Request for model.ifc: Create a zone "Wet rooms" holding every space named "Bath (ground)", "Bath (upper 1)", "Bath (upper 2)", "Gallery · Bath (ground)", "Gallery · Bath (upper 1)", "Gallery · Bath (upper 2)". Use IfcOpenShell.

First a look at what the model holds.

```python
import ifcopenshell

model = ifcopenshell.open("model.ifc")
print(model.schema)
seen = {}
for space in model.by_type("IfcSpace"):
    seen[space.Name] = seen.get(space.Name, 0) + 1
for name, count in sorted(seen.items(), key=str):
    print(count, "x", name)
print("zones:", [z.Name for z in model.by_type("IfcZone")][:20])
```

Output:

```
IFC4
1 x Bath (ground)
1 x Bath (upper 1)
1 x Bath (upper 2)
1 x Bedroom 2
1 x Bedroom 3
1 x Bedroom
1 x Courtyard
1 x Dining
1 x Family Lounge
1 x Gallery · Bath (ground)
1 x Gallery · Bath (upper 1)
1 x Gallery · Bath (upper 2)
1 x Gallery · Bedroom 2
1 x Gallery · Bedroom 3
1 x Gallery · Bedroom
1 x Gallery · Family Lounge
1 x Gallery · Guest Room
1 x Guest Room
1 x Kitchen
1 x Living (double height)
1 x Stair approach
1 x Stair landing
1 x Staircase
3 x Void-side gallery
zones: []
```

```python
import ifcopenshell
import ifcopenshell.api.group
import ifcopenshell.api.root

model = ifcopenshell.open("model.ifc")

names = {"Bath (ground)", "Bath (upper 1)", "Bath (upper 2)", "Gallery · Bath (ground)", "Gallery · Bath (upper 1)", "Gallery · Bath (upper 2)"}
spaces = [s for s in model.by_type("IfcSpace") if s.Name in names]

zone = ifcopenshell.api.root.create_entity(model, ifc_class="IfcZone", name="Wet rooms")
ifcopenshell.api.group.assign_group(model, products=spaces, group=zone)
print(len(spaces), "spaces in", zone.Name)

model.write("model-out.ifc")
```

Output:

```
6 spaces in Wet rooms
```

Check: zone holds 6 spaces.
